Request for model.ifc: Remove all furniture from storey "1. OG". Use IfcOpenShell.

First a look at what the model holds.

```python
import ifcopenshell
import ifcopenshell.util.element

model = ifcopenshell.open("model.ifc")
print(model.schema)
storey = next(s for s in model.by_type("IfcBuildingStorey") if s.Name == "1. OG")
furniture = [e for e in ifcopenshell.util.element.get_decomposition(storey) if e.is_a("IfcFurnishingElement")]
seen = {}
for e in furniture:
    element_type = ifcopenshell.util.element.get_type(e)
    name = element_type.Name if element_type not in (None, e) else None
    seen[name] = seen.get(name, 0) + 1
for name, count in sorted(seen.items(), key=str):
    print(count, "x", name)
```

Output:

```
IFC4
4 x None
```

```python
import ifcopenshell
import ifcopenshell.api.root
import ifcopenshell.util.element

model = ifcopenshell.open("model.ifc")

storey = next(s for s in model.by_type("IfcBuildingStorey") if s.Name == "1. OG")
furniture = [e for e in ifcopenshell.util.element.get_decomposition(storey) if e.is_a("IfcFurnishingElement")]

for e in furniture:
    ifcopenshell.api.root.remove_product(model, product=e)
print(len(furniture), "removed")

model.write("model_updated.ifc")
```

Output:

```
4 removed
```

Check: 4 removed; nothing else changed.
